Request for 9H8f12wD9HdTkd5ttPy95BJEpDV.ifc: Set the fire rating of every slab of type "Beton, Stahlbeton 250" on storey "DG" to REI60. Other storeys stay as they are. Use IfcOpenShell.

First a look at what the model holds.

```python
import ifcopenshell
import ifcopenshell.util.element

model = ifcopenshell.open("9H8f12wD9HdTkd5ttPy95BJEpDV.ifc")
print(model.schema)
storey = next(s for s in model.by_type("IfcBuildingStorey") if s.Name == "DG")
slabs = [e for e in ifcopenshell.util.element.get_decomposition(storey) if e.is_a("IfcSlab")]
seen = {}
for e in slabs:
    element_type = ifcopenshell.util.element.get_type(e)
    key = (element_type.Name if element_type != e and element_type else None, ifcopenshell.util.element.get_pset(e, "Pset_SlabCommon", "FireRating"))
    seen[key] = seen.get(key, 0) + 1
for (name, value), count in sorted(seen.items(), key=str):
    print(count, "x", name, "|", value)
```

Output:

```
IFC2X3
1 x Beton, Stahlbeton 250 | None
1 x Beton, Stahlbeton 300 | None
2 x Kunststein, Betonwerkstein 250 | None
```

```python
import ifcopenshell
import ifcopenshell.api.pset
import ifcopenshell.util.element

model = ifcopenshell.open("9H8f12wD9HdTkd5ttPy95BJEpDV.ifc")

storey = next(s for s in model.by_type("IfcBuildingStorey") if s.Name == "DG")
slabs = [e for e in ifcopenshell.util.element.get_decomposition(storey) if e.is_a("IfcSlab")]

count = 0
for e in slabs:
    element_type = ifcopenshell.util.element.get_type(e)
    if element_type in (None, e) or element_type.Name != "Beton, Stahlbeton 250":
        continue
    # add_pset returns the element's existing set when there is one.
    pset = ifcopenshell.api.pset.add_pset(model, product=e, name="Pset_SlabCommon")
    ifcopenshell.api.pset.edit_pset(model, pset=pset, properties={"FireRating": "REI60"})
    count += 1

print(count, "slabs updated")

model.write("9H8f12wD9HdTkd5ttPy95BJEpDV-out.ifc")
```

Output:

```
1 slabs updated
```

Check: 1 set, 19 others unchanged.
